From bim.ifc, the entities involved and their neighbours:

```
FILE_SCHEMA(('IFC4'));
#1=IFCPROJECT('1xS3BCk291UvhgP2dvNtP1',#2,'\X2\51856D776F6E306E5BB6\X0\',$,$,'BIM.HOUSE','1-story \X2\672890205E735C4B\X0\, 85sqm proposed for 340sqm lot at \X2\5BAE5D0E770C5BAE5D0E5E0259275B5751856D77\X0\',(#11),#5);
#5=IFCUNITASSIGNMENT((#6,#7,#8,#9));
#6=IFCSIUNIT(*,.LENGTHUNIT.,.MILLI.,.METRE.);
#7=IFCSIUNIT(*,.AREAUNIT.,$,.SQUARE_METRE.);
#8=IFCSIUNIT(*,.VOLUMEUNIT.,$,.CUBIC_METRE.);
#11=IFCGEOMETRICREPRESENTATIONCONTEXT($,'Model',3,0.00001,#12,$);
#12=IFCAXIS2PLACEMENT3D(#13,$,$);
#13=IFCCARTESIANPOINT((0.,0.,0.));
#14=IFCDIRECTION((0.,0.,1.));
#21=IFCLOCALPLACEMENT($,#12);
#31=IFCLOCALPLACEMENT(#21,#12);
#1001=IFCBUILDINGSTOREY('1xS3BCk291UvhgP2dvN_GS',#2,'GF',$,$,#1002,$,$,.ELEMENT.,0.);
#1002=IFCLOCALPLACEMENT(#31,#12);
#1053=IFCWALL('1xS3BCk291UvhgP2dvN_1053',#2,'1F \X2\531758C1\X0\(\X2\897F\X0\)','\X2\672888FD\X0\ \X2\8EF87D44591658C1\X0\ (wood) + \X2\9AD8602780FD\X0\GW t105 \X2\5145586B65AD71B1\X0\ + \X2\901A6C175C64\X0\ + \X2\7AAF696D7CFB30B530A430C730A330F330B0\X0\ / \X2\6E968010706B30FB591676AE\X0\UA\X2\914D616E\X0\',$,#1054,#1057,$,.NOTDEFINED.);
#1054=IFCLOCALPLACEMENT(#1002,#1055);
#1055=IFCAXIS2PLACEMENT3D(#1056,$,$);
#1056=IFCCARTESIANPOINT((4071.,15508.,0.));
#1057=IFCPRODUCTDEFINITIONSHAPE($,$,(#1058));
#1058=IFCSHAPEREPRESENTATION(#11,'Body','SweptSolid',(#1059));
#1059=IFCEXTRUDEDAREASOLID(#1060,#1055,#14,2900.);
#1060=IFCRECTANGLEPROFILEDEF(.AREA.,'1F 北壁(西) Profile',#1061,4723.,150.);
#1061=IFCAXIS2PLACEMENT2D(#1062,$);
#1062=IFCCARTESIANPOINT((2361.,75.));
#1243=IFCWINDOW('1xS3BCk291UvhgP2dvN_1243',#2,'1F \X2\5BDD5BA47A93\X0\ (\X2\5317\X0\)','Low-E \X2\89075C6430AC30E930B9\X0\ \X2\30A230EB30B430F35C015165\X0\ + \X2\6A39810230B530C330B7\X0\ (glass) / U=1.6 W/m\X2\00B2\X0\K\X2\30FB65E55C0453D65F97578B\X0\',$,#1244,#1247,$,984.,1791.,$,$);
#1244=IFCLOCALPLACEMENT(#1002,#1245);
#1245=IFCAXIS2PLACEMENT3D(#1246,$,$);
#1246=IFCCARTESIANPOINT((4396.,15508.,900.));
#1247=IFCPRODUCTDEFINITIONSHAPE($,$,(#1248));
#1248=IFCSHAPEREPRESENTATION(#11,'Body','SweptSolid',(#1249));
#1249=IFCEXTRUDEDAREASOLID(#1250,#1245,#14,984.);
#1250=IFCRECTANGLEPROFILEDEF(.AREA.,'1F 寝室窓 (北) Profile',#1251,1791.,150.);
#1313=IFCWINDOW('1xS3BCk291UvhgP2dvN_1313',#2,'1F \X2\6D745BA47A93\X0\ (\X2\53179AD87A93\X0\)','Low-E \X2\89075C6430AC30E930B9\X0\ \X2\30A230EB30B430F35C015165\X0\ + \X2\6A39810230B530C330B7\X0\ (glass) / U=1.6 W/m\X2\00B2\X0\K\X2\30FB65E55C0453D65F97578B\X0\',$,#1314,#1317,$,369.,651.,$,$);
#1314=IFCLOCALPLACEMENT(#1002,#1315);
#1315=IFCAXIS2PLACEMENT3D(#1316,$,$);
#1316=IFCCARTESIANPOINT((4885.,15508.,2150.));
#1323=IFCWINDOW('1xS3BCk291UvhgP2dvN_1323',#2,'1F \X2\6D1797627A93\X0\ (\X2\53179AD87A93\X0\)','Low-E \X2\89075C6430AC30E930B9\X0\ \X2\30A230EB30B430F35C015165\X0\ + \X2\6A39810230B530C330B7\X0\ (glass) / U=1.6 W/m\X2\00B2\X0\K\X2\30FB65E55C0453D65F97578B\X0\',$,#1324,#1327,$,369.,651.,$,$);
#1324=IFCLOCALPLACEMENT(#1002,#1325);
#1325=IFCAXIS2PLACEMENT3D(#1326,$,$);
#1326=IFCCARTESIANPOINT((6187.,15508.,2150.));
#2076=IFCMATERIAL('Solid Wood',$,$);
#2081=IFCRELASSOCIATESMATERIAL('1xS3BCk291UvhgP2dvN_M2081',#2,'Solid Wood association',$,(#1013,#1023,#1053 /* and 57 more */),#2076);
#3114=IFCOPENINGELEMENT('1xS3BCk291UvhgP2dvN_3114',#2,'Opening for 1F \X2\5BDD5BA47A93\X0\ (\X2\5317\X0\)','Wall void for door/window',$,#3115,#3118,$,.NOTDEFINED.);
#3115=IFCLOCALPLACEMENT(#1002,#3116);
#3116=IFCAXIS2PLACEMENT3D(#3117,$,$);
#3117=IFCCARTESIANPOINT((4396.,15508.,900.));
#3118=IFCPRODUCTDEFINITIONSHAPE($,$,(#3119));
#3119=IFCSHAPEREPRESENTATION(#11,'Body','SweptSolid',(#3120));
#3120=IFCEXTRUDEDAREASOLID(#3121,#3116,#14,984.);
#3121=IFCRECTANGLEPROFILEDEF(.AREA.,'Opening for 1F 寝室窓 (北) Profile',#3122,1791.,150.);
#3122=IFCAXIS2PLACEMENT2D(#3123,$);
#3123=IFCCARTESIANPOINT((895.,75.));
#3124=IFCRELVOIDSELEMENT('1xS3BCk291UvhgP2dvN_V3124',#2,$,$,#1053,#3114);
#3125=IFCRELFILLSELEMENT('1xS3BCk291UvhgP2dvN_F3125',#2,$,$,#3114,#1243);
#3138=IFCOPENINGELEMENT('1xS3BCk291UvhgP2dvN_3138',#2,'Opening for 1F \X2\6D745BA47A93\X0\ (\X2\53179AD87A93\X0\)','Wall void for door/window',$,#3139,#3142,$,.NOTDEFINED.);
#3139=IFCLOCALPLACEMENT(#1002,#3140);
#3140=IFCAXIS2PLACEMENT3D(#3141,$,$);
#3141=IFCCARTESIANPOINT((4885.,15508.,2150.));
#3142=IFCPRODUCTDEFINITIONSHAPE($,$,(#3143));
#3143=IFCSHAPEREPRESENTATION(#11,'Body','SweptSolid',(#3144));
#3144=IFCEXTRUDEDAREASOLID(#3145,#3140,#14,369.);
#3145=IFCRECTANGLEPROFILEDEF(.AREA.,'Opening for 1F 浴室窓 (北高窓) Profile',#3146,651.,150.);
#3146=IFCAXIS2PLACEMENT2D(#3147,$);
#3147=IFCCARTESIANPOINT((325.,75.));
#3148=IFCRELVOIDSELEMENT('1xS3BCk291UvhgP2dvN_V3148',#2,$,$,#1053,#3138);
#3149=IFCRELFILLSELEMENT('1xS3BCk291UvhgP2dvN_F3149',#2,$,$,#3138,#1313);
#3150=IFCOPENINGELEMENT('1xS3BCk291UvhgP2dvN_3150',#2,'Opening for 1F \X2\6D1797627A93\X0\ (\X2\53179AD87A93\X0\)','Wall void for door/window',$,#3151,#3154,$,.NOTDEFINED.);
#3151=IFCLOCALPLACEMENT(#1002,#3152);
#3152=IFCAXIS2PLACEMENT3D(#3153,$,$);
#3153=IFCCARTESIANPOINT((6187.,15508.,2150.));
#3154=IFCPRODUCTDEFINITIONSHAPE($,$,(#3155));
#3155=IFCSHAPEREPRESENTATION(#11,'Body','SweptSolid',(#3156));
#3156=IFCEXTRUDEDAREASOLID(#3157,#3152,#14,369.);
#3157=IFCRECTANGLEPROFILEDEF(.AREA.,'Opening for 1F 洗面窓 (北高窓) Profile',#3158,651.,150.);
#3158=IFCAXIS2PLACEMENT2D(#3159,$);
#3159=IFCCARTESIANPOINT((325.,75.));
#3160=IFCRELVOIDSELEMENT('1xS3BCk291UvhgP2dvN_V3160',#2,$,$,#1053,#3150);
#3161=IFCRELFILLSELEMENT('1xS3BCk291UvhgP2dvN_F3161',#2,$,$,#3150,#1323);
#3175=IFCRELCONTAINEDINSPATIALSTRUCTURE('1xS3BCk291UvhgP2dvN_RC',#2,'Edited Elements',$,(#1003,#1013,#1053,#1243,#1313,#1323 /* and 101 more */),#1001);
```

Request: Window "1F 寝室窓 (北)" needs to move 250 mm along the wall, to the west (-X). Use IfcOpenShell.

```python
import ifcopenshell
import ifcopenshell.api.geometry
import ifcopenshell.util.placement
import ifcopenshell.util.unit

model = ifcopenshell.open("bim.ifc")
unit_scale = ifcopenshell.util.unit.calculate_unit_scale(model)

window = model.by_guid("1xS3BCk291UvhgP2dvN_1243")
opening = window.FillsVoids[0].RelatingOpeningElement
wall = opening.VoidsElements[0].RelatingBuildingElement

wall_matrix = ifcopenshell.util.placement.get_local_placement(wall.ObjectPlacement)
shift = wall_matrix[:3, 0] * -0.25 / unit_scale
before = ifcopenshell.util.placement.get_local_placement(window.ObjectPlacement)[:3, 3].copy()

# The window is not placed relative to its opening, so move both.
for product in (opening, window):
    matrix = ifcopenshell.util.placement.get_local_placement(product.ObjectPlacement)
    matrix[:3, 3] += shift
    ifcopenshell.api.geometry.edit_object_placement(model, product=product, matrix=matrix, is_si=False)

after = ifcopenshell.util.placement.get_local_placement(window.ObjectPlacement)[:3, 3]
print("window moved by", (after - before).round(3) + 0.0)

model.write("bim_v2.ifc")
```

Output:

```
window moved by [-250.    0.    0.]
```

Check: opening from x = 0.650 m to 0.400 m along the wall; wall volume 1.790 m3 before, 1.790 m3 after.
